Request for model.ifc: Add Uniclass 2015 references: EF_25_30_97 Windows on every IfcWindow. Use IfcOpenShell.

First a look at what the model holds.

```python
import ifcopenshell

model = ifcopenshell.open("model.ifc")
print(model.schema)
print("classifications:", [c.Name for c in model.by_type("IfcClassification")])
for ifc_class in ("IfcDoor", "IfcRoof", "IfcStair", "IfcWall", "IfcWindow"):
    print(ifc_class, len(model.by_type(ifc_class)))
```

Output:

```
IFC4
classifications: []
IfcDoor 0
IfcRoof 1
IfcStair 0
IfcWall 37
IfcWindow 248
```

```python
import ifcopenshell
import ifcopenshell.api.classification

model = ifcopenshell.open("model.ifc")

system = ifcopenshell.api.classification.add_classification(model, classification="Uniclass 2015")

codes = {
    "IfcWindow": ("EF_25_30_97", "Windows"),
}
for ifc_class, (code, name) in codes.items():
    products = model.by_type(ifc_class)
    ifcopenshell.api.classification.add_reference(
        model, products=products, classification=system, identification=code, name=name
    )
    print(code, len(products))

model.write("model-out.ifc")
```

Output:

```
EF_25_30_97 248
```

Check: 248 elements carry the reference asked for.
